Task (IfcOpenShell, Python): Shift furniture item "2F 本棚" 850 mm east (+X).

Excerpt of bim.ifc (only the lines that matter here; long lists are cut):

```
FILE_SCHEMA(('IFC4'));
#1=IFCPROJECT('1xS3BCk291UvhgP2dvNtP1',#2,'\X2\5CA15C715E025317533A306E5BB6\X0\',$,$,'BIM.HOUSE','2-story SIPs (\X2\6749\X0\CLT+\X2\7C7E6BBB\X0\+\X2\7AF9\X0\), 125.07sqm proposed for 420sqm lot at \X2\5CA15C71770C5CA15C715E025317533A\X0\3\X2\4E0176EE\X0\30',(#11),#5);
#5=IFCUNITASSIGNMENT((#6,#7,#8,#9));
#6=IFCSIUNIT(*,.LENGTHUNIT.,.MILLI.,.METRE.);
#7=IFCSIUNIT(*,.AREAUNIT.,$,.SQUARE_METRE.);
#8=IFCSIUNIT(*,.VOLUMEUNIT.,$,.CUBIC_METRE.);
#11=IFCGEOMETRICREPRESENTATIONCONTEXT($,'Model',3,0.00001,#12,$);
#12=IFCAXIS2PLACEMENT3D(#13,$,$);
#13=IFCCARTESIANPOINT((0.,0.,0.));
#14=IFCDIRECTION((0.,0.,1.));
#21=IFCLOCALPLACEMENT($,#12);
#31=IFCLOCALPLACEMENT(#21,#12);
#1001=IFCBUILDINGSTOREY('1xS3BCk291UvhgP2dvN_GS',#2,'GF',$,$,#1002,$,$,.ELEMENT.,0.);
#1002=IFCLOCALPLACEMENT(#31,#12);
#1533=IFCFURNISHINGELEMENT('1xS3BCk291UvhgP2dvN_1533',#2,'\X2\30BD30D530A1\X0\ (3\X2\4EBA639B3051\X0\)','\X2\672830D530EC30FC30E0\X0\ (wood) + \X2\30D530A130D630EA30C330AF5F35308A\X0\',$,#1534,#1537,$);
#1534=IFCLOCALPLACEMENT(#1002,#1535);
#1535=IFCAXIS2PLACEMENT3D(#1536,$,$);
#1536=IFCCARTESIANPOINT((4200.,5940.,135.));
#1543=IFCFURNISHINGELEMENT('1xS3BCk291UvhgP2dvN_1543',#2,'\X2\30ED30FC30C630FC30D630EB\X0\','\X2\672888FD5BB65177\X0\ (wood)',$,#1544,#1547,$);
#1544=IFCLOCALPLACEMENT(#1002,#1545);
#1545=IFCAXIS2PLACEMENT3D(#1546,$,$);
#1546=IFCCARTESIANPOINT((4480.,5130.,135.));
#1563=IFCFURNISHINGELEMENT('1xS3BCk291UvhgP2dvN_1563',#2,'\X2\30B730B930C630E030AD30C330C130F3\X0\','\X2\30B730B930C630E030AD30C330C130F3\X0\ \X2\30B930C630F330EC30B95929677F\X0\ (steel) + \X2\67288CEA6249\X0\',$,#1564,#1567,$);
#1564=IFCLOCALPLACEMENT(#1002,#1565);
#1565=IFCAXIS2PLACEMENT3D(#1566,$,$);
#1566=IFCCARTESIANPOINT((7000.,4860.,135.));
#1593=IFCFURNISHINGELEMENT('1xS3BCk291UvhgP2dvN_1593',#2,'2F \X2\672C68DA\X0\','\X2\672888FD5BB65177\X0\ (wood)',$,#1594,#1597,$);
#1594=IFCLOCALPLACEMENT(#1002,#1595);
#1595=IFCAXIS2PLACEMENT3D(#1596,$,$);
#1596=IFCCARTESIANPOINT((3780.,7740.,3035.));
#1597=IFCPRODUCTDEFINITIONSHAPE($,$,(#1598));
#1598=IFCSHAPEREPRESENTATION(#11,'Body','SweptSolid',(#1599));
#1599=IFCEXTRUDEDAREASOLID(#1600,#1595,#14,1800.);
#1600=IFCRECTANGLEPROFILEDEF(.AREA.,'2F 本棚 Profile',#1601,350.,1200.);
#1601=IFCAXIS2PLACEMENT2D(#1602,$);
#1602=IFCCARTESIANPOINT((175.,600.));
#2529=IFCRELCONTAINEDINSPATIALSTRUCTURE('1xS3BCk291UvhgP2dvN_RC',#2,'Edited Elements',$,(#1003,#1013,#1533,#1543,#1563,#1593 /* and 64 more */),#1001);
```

```python
import ifcopenshell
import ifcopenshell.api.geometry
import ifcopenshell.util.placement

model = ifcopenshell.open("bim.ifc")

item = model.by_guid("1xS3BCk291UvhgP2dvN_1593")
matrix = ifcopenshell.util.placement.get_local_placement(item.ObjectPlacement)
matrix[0, 3] += 850.0
ifcopenshell.api.geometry.edit_object_placement(model, product=item, matrix=matrix, is_si=False)

print(ifcopenshell.util.placement.get_local_placement(item.ObjectPlacement).round(3) + 0.0)

model.write("bim_updated.ifc")
```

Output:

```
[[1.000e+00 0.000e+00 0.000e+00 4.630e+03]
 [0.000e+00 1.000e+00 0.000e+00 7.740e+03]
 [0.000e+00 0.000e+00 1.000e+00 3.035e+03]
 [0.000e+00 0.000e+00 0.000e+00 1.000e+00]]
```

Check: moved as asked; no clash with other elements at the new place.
